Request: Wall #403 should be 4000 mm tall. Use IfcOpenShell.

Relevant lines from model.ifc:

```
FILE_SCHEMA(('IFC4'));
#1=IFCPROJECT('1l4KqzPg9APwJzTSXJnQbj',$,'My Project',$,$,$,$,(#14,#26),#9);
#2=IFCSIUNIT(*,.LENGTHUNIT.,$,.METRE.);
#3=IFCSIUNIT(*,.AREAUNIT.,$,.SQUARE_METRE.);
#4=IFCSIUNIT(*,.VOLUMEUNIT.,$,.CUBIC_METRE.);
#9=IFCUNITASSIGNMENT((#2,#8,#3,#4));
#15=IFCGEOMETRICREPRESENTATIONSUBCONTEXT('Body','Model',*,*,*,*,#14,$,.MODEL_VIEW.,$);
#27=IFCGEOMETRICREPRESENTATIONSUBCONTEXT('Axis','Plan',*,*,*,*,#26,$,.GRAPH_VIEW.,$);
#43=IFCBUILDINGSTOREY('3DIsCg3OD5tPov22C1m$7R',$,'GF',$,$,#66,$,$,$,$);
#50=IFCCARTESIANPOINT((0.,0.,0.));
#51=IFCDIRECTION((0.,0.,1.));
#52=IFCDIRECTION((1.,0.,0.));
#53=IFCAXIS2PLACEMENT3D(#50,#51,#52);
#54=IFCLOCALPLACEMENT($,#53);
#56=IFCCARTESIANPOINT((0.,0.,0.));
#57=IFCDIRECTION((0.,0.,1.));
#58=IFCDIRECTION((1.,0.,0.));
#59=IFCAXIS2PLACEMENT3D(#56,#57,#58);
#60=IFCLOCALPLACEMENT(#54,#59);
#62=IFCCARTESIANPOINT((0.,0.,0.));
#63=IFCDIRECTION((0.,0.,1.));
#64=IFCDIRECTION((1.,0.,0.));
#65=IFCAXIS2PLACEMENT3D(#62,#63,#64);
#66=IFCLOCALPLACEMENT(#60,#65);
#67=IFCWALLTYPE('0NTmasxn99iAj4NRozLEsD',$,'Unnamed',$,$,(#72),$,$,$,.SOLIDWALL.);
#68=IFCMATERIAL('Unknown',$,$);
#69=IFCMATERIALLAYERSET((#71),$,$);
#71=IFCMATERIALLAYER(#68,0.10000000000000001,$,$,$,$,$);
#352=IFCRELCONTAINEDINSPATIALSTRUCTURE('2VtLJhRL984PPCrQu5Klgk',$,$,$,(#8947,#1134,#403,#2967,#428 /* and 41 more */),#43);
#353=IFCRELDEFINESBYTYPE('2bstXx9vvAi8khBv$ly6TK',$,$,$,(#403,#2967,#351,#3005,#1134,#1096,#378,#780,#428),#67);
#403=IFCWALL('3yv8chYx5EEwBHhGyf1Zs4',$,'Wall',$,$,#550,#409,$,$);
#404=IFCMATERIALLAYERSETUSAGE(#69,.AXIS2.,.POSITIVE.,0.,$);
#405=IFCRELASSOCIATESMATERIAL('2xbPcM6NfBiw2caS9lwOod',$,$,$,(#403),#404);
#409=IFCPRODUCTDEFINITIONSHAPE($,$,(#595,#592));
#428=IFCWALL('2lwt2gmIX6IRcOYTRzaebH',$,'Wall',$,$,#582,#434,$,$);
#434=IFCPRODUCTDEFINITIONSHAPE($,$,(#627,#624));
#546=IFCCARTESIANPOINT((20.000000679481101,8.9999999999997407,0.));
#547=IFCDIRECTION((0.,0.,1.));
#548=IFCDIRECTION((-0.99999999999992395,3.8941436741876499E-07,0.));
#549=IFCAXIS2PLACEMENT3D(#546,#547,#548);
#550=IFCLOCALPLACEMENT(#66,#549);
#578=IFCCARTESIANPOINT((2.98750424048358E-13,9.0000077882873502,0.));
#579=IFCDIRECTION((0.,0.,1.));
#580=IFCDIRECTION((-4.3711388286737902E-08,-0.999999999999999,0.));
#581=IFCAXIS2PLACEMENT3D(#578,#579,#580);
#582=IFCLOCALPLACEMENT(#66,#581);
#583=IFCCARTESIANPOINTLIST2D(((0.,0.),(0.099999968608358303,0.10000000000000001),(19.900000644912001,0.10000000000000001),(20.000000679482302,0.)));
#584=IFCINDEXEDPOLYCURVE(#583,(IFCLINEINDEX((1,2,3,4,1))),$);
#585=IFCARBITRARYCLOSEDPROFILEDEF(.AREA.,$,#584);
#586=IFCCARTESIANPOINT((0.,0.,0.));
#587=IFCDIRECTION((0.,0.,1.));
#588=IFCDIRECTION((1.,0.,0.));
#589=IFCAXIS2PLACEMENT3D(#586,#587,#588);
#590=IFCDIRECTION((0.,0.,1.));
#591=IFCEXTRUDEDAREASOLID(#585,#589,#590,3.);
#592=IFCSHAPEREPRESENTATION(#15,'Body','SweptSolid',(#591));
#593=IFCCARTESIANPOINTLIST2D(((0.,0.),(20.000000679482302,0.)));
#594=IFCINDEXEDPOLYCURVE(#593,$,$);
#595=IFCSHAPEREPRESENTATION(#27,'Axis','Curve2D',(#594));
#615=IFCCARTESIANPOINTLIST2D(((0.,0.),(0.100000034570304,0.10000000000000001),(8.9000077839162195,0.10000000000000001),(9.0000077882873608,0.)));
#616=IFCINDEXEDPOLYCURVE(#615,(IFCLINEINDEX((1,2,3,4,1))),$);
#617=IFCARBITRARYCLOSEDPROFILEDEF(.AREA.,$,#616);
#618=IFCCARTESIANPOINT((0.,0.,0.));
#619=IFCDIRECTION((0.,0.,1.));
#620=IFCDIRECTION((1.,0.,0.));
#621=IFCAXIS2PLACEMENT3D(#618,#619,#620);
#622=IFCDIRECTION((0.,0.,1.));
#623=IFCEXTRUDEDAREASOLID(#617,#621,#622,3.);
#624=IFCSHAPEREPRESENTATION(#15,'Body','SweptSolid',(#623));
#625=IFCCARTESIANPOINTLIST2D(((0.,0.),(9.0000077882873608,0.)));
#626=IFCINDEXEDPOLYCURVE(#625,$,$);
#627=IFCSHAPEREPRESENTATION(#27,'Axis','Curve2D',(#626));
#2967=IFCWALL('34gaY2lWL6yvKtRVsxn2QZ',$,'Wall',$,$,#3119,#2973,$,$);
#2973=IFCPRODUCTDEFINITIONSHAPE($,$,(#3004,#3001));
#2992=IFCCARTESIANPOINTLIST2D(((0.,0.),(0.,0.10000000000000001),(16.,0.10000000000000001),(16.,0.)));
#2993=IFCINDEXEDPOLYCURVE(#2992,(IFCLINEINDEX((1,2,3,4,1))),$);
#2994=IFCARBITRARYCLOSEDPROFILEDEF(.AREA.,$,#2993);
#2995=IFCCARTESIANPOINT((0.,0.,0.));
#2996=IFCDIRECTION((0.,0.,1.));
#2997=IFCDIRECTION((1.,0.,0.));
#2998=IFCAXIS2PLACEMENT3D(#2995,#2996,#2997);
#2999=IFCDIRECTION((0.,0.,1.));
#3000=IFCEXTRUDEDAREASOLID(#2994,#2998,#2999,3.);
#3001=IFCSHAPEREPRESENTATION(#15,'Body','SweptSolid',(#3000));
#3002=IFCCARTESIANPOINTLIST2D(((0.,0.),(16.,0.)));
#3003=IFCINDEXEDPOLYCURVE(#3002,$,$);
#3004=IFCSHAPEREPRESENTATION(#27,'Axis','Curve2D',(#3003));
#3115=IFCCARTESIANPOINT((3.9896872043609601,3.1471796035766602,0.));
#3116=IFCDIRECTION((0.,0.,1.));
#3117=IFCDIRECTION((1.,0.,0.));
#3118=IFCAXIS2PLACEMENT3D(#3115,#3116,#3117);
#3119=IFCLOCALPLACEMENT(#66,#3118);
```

```python
import ifcopenshell
import ifcopenshell.geom
import ifcopenshell.util.representation
import ifcopenshell.util.shape
import ifcopenshell.util.unit

model = ifcopenshell.open("model.ifc")
unit_scale = ifcopenshell.util.unit.calculate_unit_scale(model)
settings = ifcopenshell.geom.settings()


def volume(element):
    """Net volume in cubic metres, openings subtracted."""
    shape = ifcopenshell.geom.create_shape(settings, element)
    return ifcopenshell.util.shape.get_volume(shape.geometry)


wall = model.by_id(403)
before = volume(wall)

body = ifcopenshell.util.representation.get_representation(wall, "Model", "Body")
solid = body.Items[0]
old_height = solid.Depth
solid.Depth = 4 / unit_scale
after = volume(wall)

print(f"height {old_height:g} -> {solid.Depth:g}, volume {before:.3f} -> {after:.3f} m3")

model.write("model_rev.ifc")
```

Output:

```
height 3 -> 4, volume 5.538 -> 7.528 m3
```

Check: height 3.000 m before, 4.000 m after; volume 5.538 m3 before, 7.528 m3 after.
